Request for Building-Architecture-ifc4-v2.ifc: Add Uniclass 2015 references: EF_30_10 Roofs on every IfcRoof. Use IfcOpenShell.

First a look at what the model holds.

```python
import ifcopenshell

model = ifcopenshell.open("Building-Architecture-ifc4-v2.ifc")
print(model.schema)
print("classifications:", [c.Name for c in model.by_type("IfcClassification")])
for ifc_class in ("IfcDoor", "IfcRoof", "IfcStair", "IfcWall", "IfcWindow"):
    print(ifc_class, len(model.by_type(ifc_class)))
```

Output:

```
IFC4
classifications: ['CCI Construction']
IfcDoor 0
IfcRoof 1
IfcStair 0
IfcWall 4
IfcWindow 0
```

```python
import ifcopenshell
import ifcopenshell.api.classification

model = ifcopenshell.open("Building-Architecture-ifc4-v2.ifc")

system = ifcopenshell.api.classification.add_classification(model, classification="Uniclass 2015")

codes = {
    "IfcRoof": ("EF_30_10", "Roofs"),
}
for ifc_class, (code, name) in codes.items():
    products = model.by_type(ifc_class)
    ifcopenshell.api.classification.add_reference(
        model, products=products, classification=system, identification=code, name=name
    )
    print(code, len(products))

model.write("Building-Architecture-ifc4-v2_edited.ifc")
```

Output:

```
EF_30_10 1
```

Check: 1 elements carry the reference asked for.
